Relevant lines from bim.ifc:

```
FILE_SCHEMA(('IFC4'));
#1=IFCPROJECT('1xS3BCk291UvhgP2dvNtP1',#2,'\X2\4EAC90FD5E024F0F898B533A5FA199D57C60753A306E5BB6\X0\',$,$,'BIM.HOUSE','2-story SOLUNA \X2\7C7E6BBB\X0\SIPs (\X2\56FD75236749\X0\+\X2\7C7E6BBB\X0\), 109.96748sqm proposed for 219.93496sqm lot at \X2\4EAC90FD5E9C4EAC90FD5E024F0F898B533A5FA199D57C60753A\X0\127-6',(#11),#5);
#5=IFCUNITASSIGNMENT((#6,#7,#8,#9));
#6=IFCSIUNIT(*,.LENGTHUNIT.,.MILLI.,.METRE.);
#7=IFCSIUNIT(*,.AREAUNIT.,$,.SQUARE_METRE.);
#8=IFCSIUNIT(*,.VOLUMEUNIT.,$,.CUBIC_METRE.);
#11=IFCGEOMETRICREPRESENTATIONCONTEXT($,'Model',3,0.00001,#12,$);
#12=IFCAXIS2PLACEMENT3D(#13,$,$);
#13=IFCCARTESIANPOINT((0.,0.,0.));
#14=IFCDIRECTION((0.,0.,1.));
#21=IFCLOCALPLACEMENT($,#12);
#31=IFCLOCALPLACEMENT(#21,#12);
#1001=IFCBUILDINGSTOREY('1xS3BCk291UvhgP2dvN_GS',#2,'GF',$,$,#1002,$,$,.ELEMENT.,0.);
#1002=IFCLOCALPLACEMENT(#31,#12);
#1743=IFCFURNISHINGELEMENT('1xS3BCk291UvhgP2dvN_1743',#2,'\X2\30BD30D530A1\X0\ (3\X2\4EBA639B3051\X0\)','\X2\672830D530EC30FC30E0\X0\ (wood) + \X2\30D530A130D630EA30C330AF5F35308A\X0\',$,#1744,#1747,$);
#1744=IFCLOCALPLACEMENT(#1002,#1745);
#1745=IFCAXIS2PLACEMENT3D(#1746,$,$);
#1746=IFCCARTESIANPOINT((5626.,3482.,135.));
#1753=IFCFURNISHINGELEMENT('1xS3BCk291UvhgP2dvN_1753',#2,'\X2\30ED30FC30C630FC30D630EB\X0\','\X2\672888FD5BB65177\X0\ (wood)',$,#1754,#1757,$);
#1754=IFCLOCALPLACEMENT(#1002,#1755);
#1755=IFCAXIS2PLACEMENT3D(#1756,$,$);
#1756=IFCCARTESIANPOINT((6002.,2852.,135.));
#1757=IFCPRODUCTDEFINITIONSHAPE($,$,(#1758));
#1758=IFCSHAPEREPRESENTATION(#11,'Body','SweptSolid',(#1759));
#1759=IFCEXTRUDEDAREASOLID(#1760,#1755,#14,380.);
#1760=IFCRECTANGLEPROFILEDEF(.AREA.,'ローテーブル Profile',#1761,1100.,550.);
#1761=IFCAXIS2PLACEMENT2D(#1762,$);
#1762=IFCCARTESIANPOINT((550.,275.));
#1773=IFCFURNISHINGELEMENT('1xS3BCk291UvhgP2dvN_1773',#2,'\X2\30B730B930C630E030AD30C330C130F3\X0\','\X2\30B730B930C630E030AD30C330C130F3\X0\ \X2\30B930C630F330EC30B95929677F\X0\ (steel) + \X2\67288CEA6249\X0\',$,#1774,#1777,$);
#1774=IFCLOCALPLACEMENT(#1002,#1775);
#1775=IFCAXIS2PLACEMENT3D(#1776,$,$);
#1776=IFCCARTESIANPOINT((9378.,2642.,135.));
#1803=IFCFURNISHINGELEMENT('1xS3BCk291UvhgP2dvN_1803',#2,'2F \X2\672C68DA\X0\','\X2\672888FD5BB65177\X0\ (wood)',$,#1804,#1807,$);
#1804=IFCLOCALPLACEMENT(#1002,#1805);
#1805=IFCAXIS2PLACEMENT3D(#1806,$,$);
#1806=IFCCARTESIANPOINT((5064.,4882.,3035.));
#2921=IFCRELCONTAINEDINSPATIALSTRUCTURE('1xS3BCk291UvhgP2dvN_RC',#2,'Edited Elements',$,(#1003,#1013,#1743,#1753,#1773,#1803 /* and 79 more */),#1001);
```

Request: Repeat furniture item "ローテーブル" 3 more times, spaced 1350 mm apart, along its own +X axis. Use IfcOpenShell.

```python
import ifcopenshell
import ifcopenshell.api.geometry
import ifcopenshell.api.root
import ifcopenshell.util.element
import ifcopenshell.util.placement

model = ifcopenshell.open("bim.ifc")


def reuse_history(source, copy):
    """copy_class also copies each property set's owner history, people and application; keep the originals."""
    for rel in copy.IsDefinedBy:
        if rel.is_a("IfcRelDefinesByProperties") and (history := rel.RelatingPropertyDefinition.OwnerHistory):
            rel.RelatingPropertyDefinition.OwnerHistory = source.OwnerHistory
            ifcopenshell.util.element.remove_deep2(model, history)


source = model.by_guid("1xS3BCk291UvhgP2dvN_1753")
base = ifcopenshell.util.placement.get_local_placement(source.ObjectPlacement)
step = base[:3, 0] * 1350.0

for i in range(1, 4):
    copy = ifcopenshell.api.root.copy_class(model, product=source)
    copy.Representation = ifcopenshell.util.element.copy_deep(
        model, source.Representation, exclude=["IfcGeometricRepresentationContext", "IfcRepresentationMap"]
    )
    reuse_history(source, copy)
    matrix = base.copy()
    matrix[:3, 3] += i * step
    print("added at", matrix[:3, 3].round(3) + 0.0)
    ifcopenshell.api.geometry.edit_object_placement(model, product=copy, matrix=matrix, is_si=False)

model.write("bim_rev.ifc")
```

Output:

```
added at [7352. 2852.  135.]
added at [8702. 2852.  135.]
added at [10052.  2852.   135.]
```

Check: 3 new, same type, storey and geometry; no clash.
